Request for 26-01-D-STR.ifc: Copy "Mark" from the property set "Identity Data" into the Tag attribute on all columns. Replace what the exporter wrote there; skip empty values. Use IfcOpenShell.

First a look at what the model holds.

```python
import ifcopenshell
import ifcopenshell.util.element

model = ifcopenshell.open("26-01-D-STR.ifc")
print(model.schema)
columns = model.by_type("IfcColumn")
print(len(columns), "columns")
for e in columns[:8]:
    source = ifcopenshell.util.element.get_pset(e, "Identity Data", "Mark")
    target = e.Tag
    print(e.id(), repr(source), repr(target), sep=" | ")
```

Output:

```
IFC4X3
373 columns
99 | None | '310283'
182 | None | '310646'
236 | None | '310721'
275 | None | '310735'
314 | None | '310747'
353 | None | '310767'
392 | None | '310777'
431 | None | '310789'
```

```python
import ifcopenshell
import ifcopenshell.util.element

model = ifcopenshell.open("26-01-D-STR.ifc")

count = 0
for e in model.by_type("IfcColumn"):
    value = ifcopenshell.util.element.get_pset(e, "Identity Data", "Mark")
    current = e.Tag
    if not value or not value.strip() or current == value:
        continue
    e.Tag = value
    count += 1

print(count, "columns updated")

model.write("26-01-D-STR-out.ifc")
```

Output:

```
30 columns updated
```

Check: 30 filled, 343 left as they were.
